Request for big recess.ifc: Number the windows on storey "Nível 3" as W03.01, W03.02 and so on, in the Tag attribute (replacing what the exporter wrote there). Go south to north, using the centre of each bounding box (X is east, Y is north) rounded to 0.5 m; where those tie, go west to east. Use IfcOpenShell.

First a look at what the model holds.

```python
import ifcopenshell
import ifcopenshell.util.element
import ifcopenshell.util.placement

model = ifcopenshell.open("big recess.ifc")
print(model.schema)
storey = next(s for s in model.by_type("IfcBuildingStorey") if s.Name == "Nível 3")
windows = [e for e in ifcopenshell.util.element.get_decomposition(storey) if e.is_a("IfcWindow")]
for e in sorted(windows, key=lambda e: e.id()):
    origin = ifcopenshell.util.placement.get_local_placement(e.ObjectPlacement)[:3, 3]
    print(e.id(), e.Tag, e.Name, origin.round(2) + 0.0, sep=" | ")
```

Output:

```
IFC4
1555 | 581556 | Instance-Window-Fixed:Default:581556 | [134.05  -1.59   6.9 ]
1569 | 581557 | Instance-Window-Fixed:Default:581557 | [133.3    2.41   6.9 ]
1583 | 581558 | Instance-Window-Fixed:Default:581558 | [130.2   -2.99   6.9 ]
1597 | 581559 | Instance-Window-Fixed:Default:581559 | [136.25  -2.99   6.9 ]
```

```python
import ifcopenshell
import ifcopenshell.geom
import ifcopenshell.util.element
import ifcopenshell.util.shape

model = ifcopenshell.open("big recess.ifc")
settings = ifcopenshell.geom.settings()
settings.set("use-world-coords", True)


def centre(element):
    shape = ifcopenshell.geom.create_shape(settings, element)
    return ifcopenshell.util.shape.get_bbox_centroid(shape.geometry)


storey = next(s for s in model.by_type("IfcBuildingStorey") if s.Name == "Nível 3")
windows = [e for e in ifcopenshell.util.element.get_decomposition(storey) if e.is_a("IfcWindow")]

# Insertion points can sit at a corner or the storey origin, so sort by the geometry (in metres).
centres = {e: centre(e) for e in windows}
windows.sort(key=lambda e: (round(centres[e][1] / 0.5), centres[e][0]))

for i, e in enumerate(windows, start=1):
    number = f"W03.{i:02d}"
    e.Tag = number
    print(e.id(), number)

model.write("big recess_updated.ifc")
```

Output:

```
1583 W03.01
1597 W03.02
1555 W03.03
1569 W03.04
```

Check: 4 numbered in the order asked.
